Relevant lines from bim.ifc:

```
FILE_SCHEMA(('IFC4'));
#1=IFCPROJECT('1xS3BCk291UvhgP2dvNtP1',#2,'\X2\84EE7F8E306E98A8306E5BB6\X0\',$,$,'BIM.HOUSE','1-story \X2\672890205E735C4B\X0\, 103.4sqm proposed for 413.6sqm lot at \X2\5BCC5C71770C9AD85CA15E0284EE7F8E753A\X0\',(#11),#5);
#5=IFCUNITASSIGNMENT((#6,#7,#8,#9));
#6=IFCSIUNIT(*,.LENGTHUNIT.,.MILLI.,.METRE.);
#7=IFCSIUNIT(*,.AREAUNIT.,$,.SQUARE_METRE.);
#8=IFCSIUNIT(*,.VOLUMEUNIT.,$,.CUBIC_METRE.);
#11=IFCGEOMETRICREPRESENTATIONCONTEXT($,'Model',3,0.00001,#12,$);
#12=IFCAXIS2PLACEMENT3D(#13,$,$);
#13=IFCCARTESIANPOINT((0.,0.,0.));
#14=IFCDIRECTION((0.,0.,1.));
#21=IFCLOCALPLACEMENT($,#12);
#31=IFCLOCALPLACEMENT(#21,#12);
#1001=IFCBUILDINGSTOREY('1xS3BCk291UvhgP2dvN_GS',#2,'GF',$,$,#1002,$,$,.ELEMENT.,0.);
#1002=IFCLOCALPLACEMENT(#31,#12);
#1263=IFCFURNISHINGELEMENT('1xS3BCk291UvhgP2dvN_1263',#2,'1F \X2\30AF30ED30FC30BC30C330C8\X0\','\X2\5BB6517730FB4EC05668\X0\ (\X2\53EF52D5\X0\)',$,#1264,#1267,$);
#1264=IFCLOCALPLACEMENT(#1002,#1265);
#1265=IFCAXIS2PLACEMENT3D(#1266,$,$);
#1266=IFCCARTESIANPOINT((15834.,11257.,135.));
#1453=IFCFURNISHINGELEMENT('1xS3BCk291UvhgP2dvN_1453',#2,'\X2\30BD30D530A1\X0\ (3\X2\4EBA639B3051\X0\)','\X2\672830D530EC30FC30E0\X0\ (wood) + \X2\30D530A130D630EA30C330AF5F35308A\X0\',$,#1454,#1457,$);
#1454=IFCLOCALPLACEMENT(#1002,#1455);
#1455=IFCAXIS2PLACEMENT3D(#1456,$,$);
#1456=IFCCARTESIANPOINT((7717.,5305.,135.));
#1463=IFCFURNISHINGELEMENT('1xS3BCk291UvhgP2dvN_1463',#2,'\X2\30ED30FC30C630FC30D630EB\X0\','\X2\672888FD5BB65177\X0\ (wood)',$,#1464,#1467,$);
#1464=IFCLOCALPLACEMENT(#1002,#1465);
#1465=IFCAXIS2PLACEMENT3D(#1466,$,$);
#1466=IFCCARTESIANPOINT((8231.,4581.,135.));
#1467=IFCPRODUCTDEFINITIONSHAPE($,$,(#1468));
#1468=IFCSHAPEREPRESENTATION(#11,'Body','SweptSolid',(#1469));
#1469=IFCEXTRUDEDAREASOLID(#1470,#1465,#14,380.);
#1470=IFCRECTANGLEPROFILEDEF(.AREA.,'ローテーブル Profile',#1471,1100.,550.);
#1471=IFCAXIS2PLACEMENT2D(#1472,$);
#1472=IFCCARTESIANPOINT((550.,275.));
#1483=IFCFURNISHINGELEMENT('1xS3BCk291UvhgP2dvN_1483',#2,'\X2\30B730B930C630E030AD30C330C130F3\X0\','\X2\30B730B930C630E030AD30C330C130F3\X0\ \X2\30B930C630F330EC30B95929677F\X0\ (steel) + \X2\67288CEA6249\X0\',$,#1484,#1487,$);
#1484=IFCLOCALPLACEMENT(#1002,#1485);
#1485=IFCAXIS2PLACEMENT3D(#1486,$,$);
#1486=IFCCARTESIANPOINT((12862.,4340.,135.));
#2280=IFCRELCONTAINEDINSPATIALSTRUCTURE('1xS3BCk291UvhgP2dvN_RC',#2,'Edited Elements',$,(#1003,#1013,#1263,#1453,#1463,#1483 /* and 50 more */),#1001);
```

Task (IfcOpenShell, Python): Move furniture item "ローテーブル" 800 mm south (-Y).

```python
import ifcopenshell
import ifcopenshell.api.geometry
import ifcopenshell.util.placement

model = ifcopenshell.open("bim.ifc")

item = model.by_guid("1xS3BCk291UvhgP2dvN_1463")
matrix = ifcopenshell.util.placement.get_local_placement(item.ObjectPlacement)
matrix[1, 3] -= 800.0
ifcopenshell.api.geometry.edit_object_placement(model, product=item, matrix=matrix, is_si=False)

print(ifcopenshell.util.placement.get_local_placement(item.ObjectPlacement).round(3) + 0.0)

model.write("bim_edited.ifc")
```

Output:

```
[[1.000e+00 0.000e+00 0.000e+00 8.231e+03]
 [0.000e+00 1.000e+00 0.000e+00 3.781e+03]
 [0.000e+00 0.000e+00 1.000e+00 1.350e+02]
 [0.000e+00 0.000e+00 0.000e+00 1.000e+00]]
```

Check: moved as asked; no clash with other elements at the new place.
